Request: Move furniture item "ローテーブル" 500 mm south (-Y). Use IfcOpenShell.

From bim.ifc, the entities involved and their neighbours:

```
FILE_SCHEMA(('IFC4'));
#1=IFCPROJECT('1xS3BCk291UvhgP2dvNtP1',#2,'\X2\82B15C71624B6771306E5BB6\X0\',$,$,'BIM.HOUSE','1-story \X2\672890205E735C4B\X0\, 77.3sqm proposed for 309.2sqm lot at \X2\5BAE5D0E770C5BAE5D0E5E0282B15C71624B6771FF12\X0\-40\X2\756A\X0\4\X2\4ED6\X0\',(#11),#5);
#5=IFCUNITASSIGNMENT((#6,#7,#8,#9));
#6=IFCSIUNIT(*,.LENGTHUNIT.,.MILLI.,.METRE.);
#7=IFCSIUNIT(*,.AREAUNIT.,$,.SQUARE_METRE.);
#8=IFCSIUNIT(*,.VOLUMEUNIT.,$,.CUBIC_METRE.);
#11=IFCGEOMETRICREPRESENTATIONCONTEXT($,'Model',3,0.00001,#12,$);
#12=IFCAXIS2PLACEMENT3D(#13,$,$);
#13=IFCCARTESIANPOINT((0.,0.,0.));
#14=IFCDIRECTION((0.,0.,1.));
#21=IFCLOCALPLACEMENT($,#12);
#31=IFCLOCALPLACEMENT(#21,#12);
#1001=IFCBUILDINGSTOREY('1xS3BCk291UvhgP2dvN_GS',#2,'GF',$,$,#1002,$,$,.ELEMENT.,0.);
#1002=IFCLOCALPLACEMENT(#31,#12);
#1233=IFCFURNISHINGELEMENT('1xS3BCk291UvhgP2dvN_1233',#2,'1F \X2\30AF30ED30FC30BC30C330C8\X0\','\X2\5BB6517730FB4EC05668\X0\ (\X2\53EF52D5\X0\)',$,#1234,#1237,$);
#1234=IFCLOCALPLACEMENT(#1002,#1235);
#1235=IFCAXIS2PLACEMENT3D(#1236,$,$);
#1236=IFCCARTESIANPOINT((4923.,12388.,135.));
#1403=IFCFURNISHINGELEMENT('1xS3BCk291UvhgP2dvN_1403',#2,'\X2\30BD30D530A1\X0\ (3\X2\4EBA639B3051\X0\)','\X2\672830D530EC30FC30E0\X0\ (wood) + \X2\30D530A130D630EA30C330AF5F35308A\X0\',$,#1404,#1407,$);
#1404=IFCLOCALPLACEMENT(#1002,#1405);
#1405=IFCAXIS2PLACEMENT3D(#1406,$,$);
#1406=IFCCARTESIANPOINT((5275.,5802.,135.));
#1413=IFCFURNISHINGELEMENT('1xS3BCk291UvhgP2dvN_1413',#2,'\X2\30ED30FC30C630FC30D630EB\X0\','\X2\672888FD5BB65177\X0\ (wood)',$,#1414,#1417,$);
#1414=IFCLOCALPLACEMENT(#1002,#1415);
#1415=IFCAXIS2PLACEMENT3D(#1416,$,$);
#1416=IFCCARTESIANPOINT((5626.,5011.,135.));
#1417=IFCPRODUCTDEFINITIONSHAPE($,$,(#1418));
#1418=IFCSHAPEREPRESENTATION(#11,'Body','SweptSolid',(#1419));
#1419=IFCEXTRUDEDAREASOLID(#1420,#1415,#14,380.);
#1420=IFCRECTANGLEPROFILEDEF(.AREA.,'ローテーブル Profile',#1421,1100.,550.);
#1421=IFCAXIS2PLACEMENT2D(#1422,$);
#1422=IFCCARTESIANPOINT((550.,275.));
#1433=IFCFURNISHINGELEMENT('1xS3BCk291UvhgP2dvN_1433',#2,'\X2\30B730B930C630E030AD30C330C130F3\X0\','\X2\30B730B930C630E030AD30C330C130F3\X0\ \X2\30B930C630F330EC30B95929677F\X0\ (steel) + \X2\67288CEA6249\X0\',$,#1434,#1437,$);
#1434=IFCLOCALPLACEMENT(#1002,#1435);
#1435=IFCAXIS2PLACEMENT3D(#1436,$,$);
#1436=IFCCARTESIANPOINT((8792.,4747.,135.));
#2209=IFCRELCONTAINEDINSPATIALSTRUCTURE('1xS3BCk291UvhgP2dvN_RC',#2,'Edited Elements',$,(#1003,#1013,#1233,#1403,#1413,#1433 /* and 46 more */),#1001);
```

```python
import ifcopenshell
import ifcopenshell.api.geometry
import ifcopenshell.util.placement
import ifcopenshell.util.unit

model = ifcopenshell.open("bim.ifc")
unit_scale = ifcopenshell.util.unit.calculate_unit_scale(model)

item = model.by_guid("1xS3BCk291UvhgP2dvN_1413")
matrix = ifcopenshell.util.placement.get_local_placement(item.ObjectPlacement)
matrix[1, 3] -= 0.5 / unit_scale
ifcopenshell.api.geometry.edit_object_placement(model, product=item, matrix=matrix, is_si=False)

print(ifcopenshell.util.placement.get_local_placement(item.ObjectPlacement).round(3) + 0.0)

model.write("bim_edited.ifc")
```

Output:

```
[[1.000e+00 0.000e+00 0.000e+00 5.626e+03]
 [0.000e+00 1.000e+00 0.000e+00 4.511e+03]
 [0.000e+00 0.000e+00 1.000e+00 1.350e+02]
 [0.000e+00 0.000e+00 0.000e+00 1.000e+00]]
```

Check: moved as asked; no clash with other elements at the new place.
